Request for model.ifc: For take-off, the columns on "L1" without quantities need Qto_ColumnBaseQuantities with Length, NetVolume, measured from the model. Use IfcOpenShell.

First a look at what the model holds.

```python
import ifcopenshell
import ifcopenshell.util.element
import ifcopenshell.util.unit

model = ifcopenshell.open("model.ifc")
print(model.schema)
for unit_type in ("LENGTHUNIT", "AREAUNIT", "VOLUMEUNIT"):
    print(unit_type, ifcopenshell.util.unit.calculate_unit_scale(model, unit_type))
storey = next(s for s in model.by_type("IfcBuildingStorey") if s.Name == "L1")
columns = [e for e in ifcopenshell.util.element.get_decomposition(storey) if e.is_a("IfcColumn")]
for e in sorted(columns, key=lambda e: e.id()):
    print(e.id(), e.is_a(), e.Name, list(ifcopenshell.util.element.get_psets(e, qtos_only=True)), sep=" | ")
```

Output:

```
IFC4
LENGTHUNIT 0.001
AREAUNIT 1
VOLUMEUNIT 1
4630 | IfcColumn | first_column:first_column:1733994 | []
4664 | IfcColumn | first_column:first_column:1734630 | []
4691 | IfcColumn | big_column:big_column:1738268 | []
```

```python
import ifcopenshell
import ifcopenshell.api.pset
import ifcopenshell.geom
import ifcopenshell.util.element
import ifcopenshell.util.shape
import ifcopenshell.util.unit

model = ifcopenshell.open("model.ifc")
unit_scale = ifcopenshell.util.unit.calculate_unit_scale(model)
volume_scale = ifcopenshell.util.unit.calculate_unit_scale(model, "VOLUMEUNIT")
settings = ifcopenshell.geom.settings()

storey = next(s for s in model.by_type("IfcBuildingStorey") if s.Name == "L1")
columns = [e for e in ifcopenshell.util.element.get_decomposition(storey) if e.is_a("IfcColumn")]

for e in sorted(columns, key=lambda e: e.id()):
    if ifcopenshell.util.element.get_psets(e, qtos_only=True, should_inherit=False):
        continue
    # Geometry comes back in metres, in the element's own axes.
    shape = ifcopenshell.geom.create_shape(settings, e)
    values = {
        "Length": ifcopenshell.util.shape.get_z(shape.geometry) / unit_scale,
        "NetVolume": ifcopenshell.util.shape.get_volume(shape.geometry) / volume_scale,
    }
    qto = ifcopenshell.api.pset.add_qto(model, product=e, name="Qto_ColumnBaseQuantities")
    ifcopenshell.api.pset.edit_qto(model, qto=qto, properties=values)
    print(e.id(), {k: round(v, 3) for k, v in values.items()})

model.write("model_v2.ifc")
```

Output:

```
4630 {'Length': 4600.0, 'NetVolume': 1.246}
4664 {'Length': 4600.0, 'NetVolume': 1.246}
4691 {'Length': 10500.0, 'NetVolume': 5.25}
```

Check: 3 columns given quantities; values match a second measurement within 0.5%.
